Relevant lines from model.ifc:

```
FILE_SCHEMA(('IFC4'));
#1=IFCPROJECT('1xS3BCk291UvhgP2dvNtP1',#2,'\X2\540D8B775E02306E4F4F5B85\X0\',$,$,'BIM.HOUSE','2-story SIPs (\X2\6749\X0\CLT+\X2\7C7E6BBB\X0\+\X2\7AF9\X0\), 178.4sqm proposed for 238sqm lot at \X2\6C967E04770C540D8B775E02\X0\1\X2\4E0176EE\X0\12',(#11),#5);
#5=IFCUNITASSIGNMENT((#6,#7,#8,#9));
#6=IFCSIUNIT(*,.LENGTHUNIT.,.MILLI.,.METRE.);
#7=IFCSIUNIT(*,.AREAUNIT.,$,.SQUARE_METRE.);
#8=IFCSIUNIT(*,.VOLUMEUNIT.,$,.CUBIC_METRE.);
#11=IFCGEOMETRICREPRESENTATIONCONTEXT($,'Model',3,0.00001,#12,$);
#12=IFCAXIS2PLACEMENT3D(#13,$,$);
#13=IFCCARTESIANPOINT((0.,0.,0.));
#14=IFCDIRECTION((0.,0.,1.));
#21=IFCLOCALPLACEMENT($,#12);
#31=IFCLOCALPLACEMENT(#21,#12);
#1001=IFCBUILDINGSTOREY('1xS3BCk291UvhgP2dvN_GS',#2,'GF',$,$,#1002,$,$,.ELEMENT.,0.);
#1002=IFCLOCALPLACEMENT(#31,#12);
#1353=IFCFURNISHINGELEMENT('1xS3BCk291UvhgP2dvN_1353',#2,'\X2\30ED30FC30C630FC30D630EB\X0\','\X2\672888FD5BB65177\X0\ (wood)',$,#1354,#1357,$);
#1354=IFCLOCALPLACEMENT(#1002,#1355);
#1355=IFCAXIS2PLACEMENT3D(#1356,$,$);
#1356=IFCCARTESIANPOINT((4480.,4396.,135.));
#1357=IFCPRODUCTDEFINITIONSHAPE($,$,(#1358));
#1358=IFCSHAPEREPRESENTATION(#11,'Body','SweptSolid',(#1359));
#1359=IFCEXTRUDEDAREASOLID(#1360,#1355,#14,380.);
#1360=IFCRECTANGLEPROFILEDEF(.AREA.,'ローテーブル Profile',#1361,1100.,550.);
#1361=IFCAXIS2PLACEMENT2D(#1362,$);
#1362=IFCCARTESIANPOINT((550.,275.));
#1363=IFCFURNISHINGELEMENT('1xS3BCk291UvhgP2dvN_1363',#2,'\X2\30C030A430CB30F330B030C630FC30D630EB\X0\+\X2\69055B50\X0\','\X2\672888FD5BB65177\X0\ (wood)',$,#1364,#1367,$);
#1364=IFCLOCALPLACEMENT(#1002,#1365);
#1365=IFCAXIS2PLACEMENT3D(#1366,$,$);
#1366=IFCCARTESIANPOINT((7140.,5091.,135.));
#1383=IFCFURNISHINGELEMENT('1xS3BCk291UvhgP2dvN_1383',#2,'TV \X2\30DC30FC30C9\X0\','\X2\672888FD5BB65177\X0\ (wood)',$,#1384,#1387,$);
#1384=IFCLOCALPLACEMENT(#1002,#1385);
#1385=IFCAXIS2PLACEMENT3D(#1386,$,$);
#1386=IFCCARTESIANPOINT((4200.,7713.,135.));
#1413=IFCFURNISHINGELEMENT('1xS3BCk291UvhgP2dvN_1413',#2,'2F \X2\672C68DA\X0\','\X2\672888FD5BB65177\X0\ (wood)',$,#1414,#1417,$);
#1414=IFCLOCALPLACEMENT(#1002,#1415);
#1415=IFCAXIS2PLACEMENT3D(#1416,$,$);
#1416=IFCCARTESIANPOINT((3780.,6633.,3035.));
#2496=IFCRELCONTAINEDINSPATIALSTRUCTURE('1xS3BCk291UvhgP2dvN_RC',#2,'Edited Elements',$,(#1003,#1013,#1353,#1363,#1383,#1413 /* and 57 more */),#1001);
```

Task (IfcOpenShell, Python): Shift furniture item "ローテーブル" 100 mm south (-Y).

```python
import ifcopenshell
import ifcopenshell.api.geometry
import ifcopenshell.util.placement
import ifcopenshell.util.unit

model = ifcopenshell.open("model.ifc")
unit_scale = ifcopenshell.util.unit.calculate_unit_scale(model)

item = model.by_id(1353)
matrix = ifcopenshell.util.placement.get_local_placement(item.ObjectPlacement)
matrix[1, 3] -= 0.1 / unit_scale
ifcopenshell.api.geometry.edit_object_placement(model, product=item, matrix=matrix, is_si=False)

print(ifcopenshell.util.placement.get_local_placement(item.ObjectPlacement).round(3) + 0.0)

model.write("model_updated.ifc")
```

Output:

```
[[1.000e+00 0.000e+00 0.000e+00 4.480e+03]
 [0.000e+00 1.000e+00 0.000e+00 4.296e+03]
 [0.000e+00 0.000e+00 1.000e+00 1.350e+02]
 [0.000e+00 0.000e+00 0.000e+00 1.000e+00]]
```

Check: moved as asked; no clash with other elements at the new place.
